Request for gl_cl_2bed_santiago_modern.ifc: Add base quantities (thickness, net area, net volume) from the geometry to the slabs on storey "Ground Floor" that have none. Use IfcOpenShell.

First a look at what the model holds.

```python
import ifcopenshell
import ifcopenshell.util.element
import ifcopenshell.util.unit

model = ifcopenshell.open("gl_cl_2bed_santiago_modern.ifc")
print(model.schema)
for unit_type in ("LENGTHUNIT", "AREAUNIT", "VOLUMEUNIT"):
    print(unit_type, ifcopenshell.util.unit.calculate_unit_scale(model, unit_type))
storey = next(s for s in model.by_type("IfcBuildingStorey") if s.Name == "Ground Floor")
slabs = [e for e in ifcopenshell.util.element.get_decomposition(storey) if e.is_a("IfcSlab")]
for e in sorted(slabs, key=lambda e: e.id()):
    print(e.id(), e.is_a(), e.Name, list(ifcopenshell.util.element.get_psets(e, qtos_only=True)), sep=" | ")
```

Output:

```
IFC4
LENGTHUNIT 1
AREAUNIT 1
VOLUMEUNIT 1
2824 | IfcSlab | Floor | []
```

```python
import ifcopenshell
import ifcopenshell.api.pset
import ifcopenshell.geom
import ifcopenshell.util.element
import ifcopenshell.util.shape
import ifcopenshell.util.unit

model = ifcopenshell.open("gl_cl_2bed_santiago_modern.ifc")
unit_scale = ifcopenshell.util.unit.calculate_unit_scale(model)
area_scale = ifcopenshell.util.unit.calculate_unit_scale(model, "AREAUNIT")
volume_scale = ifcopenshell.util.unit.calculate_unit_scale(model, "VOLUMEUNIT")
settings = ifcopenshell.geom.settings()

storey = next(s for s in model.by_type("IfcBuildingStorey") if s.Name == "Ground Floor")
slabs = [e for e in ifcopenshell.util.element.get_decomposition(storey) if e.is_a("IfcSlab")]

for e in sorted(slabs, key=lambda e: e.id()):
    if ifcopenshell.util.element.get_psets(e, qtos_only=True, should_inherit=False):
        continue
    # Geometry comes back in metres, in the element's own axes.
    shape = ifcopenshell.geom.create_shape(settings, e)
    values = {
        "Width": ifcopenshell.util.shape.get_z(shape.geometry) / unit_scale,
        "NetArea": ifcopenshell.util.shape.get_footprint_area(shape.geometry) / area_scale,
        "NetVolume": ifcopenshell.util.shape.get_volume(shape.geometry) / volume_scale,
    }
    qto = ifcopenshell.api.pset.add_qto(model, product=e, name="Qto_SlabBaseQuantities")
    ifcopenshell.api.pset.edit_qto(model, qto=qto, properties=values)
    print(e.id(), {k: round(v, 3) for k, v in values.items()})

model.write("gl_cl_2bed_santiago_modern_v2.ifc")
```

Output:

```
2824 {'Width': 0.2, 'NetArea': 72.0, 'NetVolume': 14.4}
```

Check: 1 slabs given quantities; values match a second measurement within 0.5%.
